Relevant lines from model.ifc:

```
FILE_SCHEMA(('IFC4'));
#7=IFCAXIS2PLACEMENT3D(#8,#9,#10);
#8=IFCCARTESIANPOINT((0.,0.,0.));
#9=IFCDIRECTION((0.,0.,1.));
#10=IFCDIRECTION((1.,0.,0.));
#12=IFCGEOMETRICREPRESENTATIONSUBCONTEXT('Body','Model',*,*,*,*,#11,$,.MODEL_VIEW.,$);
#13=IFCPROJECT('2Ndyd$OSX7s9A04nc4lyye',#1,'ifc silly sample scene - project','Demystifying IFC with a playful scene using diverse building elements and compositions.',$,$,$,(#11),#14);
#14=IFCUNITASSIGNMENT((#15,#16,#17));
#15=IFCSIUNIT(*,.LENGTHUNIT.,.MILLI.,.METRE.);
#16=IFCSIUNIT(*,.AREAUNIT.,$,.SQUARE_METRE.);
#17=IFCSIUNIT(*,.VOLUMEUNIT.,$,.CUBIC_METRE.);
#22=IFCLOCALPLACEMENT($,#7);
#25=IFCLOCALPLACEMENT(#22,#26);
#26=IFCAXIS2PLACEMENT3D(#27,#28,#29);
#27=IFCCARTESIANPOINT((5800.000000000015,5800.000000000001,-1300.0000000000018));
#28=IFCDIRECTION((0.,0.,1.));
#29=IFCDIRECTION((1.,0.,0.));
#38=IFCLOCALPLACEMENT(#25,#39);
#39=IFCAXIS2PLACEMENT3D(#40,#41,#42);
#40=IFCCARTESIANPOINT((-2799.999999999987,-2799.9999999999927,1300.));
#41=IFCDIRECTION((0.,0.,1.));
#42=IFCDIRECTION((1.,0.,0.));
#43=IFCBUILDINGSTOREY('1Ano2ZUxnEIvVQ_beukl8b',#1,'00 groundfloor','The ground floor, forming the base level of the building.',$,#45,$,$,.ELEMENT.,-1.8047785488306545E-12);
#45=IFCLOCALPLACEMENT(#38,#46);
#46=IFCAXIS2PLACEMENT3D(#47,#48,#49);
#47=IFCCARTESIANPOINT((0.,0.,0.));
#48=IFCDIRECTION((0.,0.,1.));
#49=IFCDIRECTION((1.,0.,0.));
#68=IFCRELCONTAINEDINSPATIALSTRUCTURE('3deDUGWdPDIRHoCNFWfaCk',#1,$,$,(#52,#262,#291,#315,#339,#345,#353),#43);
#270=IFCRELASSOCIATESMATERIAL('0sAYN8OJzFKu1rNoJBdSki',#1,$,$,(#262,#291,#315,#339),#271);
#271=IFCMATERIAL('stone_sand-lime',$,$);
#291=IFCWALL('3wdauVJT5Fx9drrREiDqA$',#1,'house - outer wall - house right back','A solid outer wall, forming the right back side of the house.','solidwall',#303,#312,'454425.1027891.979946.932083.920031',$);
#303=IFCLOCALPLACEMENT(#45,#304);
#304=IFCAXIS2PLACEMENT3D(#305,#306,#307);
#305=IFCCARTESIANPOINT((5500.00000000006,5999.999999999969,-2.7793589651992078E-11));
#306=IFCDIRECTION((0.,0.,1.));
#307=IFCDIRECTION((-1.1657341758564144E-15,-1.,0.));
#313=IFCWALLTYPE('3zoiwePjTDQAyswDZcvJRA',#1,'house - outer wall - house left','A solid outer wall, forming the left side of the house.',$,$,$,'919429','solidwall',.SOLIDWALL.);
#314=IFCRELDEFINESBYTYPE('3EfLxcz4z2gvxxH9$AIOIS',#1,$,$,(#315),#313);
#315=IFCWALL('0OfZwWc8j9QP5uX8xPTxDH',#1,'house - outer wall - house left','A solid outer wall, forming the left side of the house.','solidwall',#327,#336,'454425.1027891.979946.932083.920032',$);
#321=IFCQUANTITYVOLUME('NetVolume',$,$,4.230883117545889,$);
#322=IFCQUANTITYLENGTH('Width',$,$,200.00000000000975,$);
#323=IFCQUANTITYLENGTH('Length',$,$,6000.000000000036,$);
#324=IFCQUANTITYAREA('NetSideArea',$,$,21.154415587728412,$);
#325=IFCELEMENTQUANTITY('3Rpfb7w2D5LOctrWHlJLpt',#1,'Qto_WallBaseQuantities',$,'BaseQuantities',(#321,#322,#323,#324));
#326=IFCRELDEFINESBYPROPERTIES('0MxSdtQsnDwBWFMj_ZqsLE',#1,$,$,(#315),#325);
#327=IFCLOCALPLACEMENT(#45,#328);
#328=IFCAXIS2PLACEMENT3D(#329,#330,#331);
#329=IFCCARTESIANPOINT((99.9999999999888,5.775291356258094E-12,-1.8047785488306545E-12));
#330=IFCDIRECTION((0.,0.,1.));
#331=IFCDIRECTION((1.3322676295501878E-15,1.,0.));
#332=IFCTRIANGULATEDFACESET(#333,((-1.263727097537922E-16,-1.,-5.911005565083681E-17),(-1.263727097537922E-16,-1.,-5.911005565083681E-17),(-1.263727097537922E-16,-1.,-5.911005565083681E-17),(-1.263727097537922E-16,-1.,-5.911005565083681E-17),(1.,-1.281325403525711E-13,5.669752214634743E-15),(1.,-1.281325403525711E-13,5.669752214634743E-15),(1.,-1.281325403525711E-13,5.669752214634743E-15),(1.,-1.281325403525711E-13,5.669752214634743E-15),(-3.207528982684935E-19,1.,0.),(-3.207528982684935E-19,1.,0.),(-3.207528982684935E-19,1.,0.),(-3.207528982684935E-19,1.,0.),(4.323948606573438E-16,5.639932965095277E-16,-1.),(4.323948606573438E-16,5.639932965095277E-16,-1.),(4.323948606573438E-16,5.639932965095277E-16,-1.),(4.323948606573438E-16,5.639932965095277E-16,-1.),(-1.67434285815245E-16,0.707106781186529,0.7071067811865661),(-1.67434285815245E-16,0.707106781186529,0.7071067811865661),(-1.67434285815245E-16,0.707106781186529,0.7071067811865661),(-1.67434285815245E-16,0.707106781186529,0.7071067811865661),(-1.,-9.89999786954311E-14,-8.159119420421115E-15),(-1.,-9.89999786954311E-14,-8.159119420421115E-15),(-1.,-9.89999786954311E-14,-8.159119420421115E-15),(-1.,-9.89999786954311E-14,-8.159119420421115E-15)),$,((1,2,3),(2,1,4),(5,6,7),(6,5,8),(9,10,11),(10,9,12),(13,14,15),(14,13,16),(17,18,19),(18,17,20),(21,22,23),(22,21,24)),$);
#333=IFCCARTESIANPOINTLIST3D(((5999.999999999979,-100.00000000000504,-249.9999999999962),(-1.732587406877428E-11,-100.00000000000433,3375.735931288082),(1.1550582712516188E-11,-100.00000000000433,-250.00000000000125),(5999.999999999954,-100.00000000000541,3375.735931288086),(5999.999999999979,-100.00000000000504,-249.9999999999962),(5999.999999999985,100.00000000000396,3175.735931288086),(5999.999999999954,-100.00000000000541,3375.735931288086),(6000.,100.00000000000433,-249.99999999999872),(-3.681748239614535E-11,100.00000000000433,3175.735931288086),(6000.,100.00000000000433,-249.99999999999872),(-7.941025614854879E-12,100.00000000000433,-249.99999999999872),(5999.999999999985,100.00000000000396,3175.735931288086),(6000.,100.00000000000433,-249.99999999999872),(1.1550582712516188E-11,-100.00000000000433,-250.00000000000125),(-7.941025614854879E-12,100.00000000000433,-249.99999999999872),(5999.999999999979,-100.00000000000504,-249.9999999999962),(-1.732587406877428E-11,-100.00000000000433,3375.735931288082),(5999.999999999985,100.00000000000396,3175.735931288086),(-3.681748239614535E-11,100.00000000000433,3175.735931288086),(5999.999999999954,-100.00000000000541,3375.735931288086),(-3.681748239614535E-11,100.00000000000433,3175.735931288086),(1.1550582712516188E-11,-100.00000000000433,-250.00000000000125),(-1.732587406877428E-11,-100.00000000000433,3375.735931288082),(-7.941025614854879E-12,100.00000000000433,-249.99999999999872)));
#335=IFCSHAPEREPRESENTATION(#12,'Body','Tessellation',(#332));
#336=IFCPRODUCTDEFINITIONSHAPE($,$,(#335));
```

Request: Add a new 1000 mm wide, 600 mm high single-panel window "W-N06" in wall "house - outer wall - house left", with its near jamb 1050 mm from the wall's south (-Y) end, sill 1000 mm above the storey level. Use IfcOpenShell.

```python
import numpy as np
import ifcopenshell
import ifcopenshell.api.feature
import ifcopenshell.api.geometry
import ifcopenshell.api.pset
import ifcopenshell.api.root
import ifcopenshell.api.spatial
import ifcopenshell.geom
import ifcopenshell.util.element
import ifcopenshell.util.placement
import ifcopenshell.util.representation
import ifcopenshell.util.shape
import ifcopenshell.util.unit

model = ifcopenshell.open("model.ifc")
unit_scale = ifcopenshell.util.unit.calculate_unit_scale(model)
area_scale = ifcopenshell.util.unit.calculate_unit_scale(model, "AREAUNIT")
volume_scale = ifcopenshell.util.unit.calculate_unit_scale(model, "VOLUMEUNIT")
settings = ifcopenshell.geom.settings()


def volume(element):
    """Net volume in cubic metres, openings subtracted."""
    shape = ifcopenshell.geom.create_shape(settings, element)
    return ifcopenshell.util.shape.get_volume(shape.geometry)


wall = model.by_guid("0OfZwWc8j9QP5uX8xPTxDH")
storey = ifcopenshell.util.element.get_container(wall, ifc_class="IfcBuildingStorey")
context = ifcopenshell.util.representation.get_context(model, "Model", "Body", "MODEL_VIEW")
before = volume(wall)

width, height, from_end, sill = 1, 0.6, 1.05, 1  # metres

# The wall runs along its own X axis, and the end named is its -X end.
wall_shape = ifcopenshell.geom.create_shape(settings, wall)
x, y, z = ifcopenshell.util.shape.get_vertices(wall_shape.geometry).T
start = x.min() + from_end
face, thickness = float(y.min()), float(y.max() - y.min())
wall_matrix = ifcopenshell.util.placement.get_local_placement(wall.ObjectPlacement)
level = ifcopenshell.util.placement.get_local_placement(storey.ObjectPlacement)[2, 3]


def in_wall(x, y):
    """Placement at x, y metres in the wall's axes, at sill height."""
    matrix = wall_matrix.copy()
    matrix[:, 3] = wall_matrix @ np.array([x / unit_scale, y / unit_scale, 0.0, 1.0])
    matrix[2, 3] = level + sill / unit_scale
    return matrix


# Opening: a box that overshoots both wall faces by 50 mm.
opening = ifcopenshell.api.root.create_entity(model, ifc_class="IfcOpeningElement", predefined_type="OPENING")
box = ifcopenshell.api.geometry.add_wall_representation(
    model, context=context, length=width, height=height, thickness=thickness + 0.1
)
ifcopenshell.api.geometry.assign_representation(model, product=opening, representation=box)
ifcopenshell.api.geometry.edit_object_placement(model, product=opening, matrix=in_wall(start, face - 0.05), is_si=False)
ifcopenshell.api.feature.add_feature(model, feature=opening, element=wall)

window = ifcopenshell.api.root.create_entity(model, ifc_class="IfcWindow", name="W-N06", predefined_type="WINDOW")
window.OverallWidth, window.OverallHeight = width / unit_scale, height / unit_scale
window.PartitioningType = "SINGLE_PANEL"
body = ifcopenshell.api.geometry.add_window_representation(
    model,
    context=context,
    overall_width=window.OverallWidth,
    overall_height=window.OverallHeight,
    partition_type="SINGLE_PANEL",
)
ifcopenshell.api.geometry.assign_representation(model, product=window, representation=body)
ifcopenshell.api.spatial.assign_container(model, products=[window], relating_structure=storey)
ifcopenshell.api.feature.add_filling(model, opening=opening, element=window)

# Centre the window in the wall's thickness.
ifcopenshell.api.geometry.edit_object_placement(model, product=window, matrix=in_wall(start, face), is_si=False)
window_shape = ifcopenshell.geom.create_shape(settings, window)
depth = ifcopenshell.util.shape.get_vertices(window_shape.geometry)[:, 1]
offset = face + thickness / 2 - (depth.min() + depth.max()) / 2
ifcopenshell.api.geometry.edit_object_placement(model, product=window, matrix=in_wall(start, offset), is_si=False)

after = volume(wall)

# Update the wall's stored quantities.
qto = model.by_id(ifcopenshell.util.element.get_pset(wall, "Qto_WallBaseQuantities", should_inherit=False)["id"])
ifcopenshell.api.pset.edit_qto(model, qto=qto, properties={
    "NetVolume": after / volume_scale,
    "NetSideArea": after / thickness / area_scale,
})

print(f"wall volume {before:.3f} -> {after:.3f} m3")

model.write("model_edited.ifc")
```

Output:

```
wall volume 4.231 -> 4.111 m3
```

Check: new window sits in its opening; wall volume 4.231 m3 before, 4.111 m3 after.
